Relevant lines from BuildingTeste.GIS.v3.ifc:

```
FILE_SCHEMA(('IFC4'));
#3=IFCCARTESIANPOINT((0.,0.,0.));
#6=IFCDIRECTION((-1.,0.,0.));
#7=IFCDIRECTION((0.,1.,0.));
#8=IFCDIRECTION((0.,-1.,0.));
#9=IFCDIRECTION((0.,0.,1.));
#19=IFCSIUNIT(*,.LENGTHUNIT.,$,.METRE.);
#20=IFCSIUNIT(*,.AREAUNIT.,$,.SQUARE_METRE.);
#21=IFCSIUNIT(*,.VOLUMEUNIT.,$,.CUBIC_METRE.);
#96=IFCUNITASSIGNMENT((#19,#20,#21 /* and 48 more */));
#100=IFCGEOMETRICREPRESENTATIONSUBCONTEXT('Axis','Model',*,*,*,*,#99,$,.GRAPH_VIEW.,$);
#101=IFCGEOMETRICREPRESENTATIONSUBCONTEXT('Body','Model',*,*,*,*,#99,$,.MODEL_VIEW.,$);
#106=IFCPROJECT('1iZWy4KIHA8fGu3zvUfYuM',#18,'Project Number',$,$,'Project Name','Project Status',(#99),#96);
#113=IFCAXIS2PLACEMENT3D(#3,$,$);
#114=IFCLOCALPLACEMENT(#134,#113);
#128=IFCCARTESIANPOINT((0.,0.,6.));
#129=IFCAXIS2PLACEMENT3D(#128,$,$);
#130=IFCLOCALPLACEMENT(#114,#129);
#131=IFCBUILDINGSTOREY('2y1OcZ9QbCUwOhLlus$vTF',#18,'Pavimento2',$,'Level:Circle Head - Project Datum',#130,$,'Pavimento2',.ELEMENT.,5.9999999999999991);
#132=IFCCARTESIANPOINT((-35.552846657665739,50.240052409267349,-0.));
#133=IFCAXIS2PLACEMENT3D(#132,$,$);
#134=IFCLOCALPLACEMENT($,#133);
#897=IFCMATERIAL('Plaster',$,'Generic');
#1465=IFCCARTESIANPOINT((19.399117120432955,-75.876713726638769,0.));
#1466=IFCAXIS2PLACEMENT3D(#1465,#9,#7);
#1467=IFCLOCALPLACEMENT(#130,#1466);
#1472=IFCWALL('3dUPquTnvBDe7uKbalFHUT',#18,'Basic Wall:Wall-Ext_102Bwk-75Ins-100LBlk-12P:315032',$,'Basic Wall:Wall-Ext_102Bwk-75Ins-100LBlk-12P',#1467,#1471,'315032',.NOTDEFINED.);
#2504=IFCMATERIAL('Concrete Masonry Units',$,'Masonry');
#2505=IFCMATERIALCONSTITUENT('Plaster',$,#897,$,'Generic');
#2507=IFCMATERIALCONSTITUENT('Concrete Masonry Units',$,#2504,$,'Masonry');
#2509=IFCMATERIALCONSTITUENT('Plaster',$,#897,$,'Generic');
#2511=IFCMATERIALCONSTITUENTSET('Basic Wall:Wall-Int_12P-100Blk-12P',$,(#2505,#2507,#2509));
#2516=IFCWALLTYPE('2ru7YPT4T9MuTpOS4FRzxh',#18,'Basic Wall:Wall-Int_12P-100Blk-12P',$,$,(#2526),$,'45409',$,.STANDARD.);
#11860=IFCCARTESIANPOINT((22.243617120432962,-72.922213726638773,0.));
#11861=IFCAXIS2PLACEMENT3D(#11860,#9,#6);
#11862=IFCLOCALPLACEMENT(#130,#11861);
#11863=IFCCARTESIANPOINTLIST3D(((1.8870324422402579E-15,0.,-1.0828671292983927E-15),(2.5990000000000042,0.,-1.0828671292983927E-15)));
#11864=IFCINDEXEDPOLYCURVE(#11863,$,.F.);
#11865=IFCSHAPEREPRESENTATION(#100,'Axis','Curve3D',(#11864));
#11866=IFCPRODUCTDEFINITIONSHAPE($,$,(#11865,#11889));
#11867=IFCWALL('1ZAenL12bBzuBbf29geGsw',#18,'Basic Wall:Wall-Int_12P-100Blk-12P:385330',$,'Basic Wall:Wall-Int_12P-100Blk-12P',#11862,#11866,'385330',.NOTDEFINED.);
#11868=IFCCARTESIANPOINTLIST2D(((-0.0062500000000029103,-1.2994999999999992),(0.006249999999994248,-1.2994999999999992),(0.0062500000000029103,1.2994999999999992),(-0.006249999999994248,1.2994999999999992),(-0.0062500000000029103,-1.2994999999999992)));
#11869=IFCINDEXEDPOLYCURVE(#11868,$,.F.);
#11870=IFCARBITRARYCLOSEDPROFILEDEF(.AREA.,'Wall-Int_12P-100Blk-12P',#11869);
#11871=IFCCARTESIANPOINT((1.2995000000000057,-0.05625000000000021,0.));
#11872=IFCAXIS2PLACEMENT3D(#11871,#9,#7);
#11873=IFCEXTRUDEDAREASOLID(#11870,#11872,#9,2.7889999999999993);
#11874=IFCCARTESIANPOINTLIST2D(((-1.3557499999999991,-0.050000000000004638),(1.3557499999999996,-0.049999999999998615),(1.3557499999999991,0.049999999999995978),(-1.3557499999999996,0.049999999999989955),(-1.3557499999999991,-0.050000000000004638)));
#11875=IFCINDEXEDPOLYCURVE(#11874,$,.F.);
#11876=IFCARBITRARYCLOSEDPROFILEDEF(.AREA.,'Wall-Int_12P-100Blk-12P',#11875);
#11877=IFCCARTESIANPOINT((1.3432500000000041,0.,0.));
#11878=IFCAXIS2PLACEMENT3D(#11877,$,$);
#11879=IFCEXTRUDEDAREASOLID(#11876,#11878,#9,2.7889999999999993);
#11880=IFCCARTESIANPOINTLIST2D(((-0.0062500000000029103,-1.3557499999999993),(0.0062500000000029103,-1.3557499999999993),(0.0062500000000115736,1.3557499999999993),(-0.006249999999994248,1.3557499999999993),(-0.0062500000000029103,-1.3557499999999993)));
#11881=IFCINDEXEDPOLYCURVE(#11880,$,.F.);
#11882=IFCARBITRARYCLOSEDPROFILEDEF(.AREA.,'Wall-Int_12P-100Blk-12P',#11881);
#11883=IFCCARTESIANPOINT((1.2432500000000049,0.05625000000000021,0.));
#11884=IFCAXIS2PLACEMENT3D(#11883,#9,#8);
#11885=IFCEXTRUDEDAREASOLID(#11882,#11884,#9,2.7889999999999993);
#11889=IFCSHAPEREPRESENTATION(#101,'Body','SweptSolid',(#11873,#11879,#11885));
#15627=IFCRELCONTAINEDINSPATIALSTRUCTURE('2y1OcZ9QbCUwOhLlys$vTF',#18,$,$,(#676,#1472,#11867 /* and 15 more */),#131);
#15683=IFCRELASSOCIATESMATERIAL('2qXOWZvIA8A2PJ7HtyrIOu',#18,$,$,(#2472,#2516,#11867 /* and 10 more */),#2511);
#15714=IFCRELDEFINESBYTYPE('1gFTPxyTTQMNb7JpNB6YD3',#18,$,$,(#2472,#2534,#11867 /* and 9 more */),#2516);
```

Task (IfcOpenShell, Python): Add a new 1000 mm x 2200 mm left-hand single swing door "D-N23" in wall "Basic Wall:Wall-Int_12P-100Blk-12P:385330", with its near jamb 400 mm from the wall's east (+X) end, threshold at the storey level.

```python
import numpy as np
import ifcopenshell
import ifcopenshell.api.feature
import ifcopenshell.api.geometry
import ifcopenshell.api.root
import ifcopenshell.api.spatial
import ifcopenshell.geom
import ifcopenshell.util.element
import ifcopenshell.util.placement
import ifcopenshell.util.representation
import ifcopenshell.util.shape
import ifcopenshell.util.unit

model = ifcopenshell.open("BuildingTeste.GIS.v3.ifc")
unit_scale = ifcopenshell.util.unit.calculate_unit_scale(model)
settings = ifcopenshell.geom.settings()


def volume(element):
    """Net volume in cubic metres, openings subtracted."""
    shape = ifcopenshell.geom.create_shape(settings, element)
    return ifcopenshell.util.shape.get_volume(shape.geometry)


wall = model.by_guid("1ZAenL12bBzuBbf29geGsw")
storey = ifcopenshell.util.element.get_container(wall, ifc_class="IfcBuildingStorey")
context = ifcopenshell.util.representation.get_context(model, "Model", "Body", "MODEL_VIEW")
before = volume(wall)

width, height, from_end, sill = 1, 2.2, 0.4, 0.0  # metres

# The wall runs along its own X axis, and the end named is its -X end.
wall_shape = ifcopenshell.geom.create_shape(settings, wall)
x, y, z = ifcopenshell.util.shape.get_vertices(wall_shape.geometry).T
start = x.min() + from_end
face, thickness = float(y.min()), float(y.max() - y.min())
wall_matrix = ifcopenshell.util.placement.get_local_placement(wall.ObjectPlacement)
level = ifcopenshell.util.placement.get_local_placement(storey.ObjectPlacement)[2, 3]


def in_wall(x, y):
    """Placement at x, y metres in the wall's axes, at sill height."""
    matrix = wall_matrix.copy()
    matrix[:, 3] = wall_matrix @ np.array([x / unit_scale, y / unit_scale, 0.0, 1.0])
    matrix[2, 3] = level + sill / unit_scale
    return matrix


# Opening: a box that overshoots both wall faces by 50 mm.
opening = ifcopenshell.api.root.create_entity(model, ifc_class="IfcOpeningElement", predefined_type="OPENING")
box = ifcopenshell.api.geometry.add_wall_representation(
    model, context=context, length=width, height=height, thickness=thickness + 0.1
)
ifcopenshell.api.geometry.assign_representation(model, product=opening, representation=box)
ifcopenshell.api.geometry.edit_object_placement(model, product=opening, matrix=in_wall(start, face - 0.05), is_si=False)
ifcopenshell.api.feature.add_feature(model, feature=opening, element=wall)

door = ifcopenshell.api.root.create_entity(model, ifc_class="IfcDoor", name="D-N23", predefined_type="DOOR")
door.OverallWidth, door.OverallHeight = width / unit_scale, height / unit_scale
door.OperationType = "SINGLE_SWING_LEFT"
body = ifcopenshell.api.geometry.add_door_representation(
    model,
    context=context,
    overall_width=door.OverallWidth,
    overall_height=door.OverallHeight,
    operation_type="SINGLE_SWING_LEFT",
    lining_properties={"LiningDepth": thickness / unit_scale, "ThresholdDepth": thickness / unit_scale},
)
ifcopenshell.api.geometry.assign_representation(model, product=door, representation=body)
ifcopenshell.api.spatial.assign_container(model, products=[door], relating_structure=storey)
ifcopenshell.api.feature.add_filling(model, opening=opening, element=door)

# The lining spans the wall, so the door starts at the wall face.
ifcopenshell.api.geometry.edit_object_placement(model, product=door, matrix=in_wall(start, face), is_si=False)

after = volume(wall)

print(f"wall volume {before:.3f} -> {after:.3f} m3")

model.write("BuildingTeste.GIS.v3_edited.ifc")
```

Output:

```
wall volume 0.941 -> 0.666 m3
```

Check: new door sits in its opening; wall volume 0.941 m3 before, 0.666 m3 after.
